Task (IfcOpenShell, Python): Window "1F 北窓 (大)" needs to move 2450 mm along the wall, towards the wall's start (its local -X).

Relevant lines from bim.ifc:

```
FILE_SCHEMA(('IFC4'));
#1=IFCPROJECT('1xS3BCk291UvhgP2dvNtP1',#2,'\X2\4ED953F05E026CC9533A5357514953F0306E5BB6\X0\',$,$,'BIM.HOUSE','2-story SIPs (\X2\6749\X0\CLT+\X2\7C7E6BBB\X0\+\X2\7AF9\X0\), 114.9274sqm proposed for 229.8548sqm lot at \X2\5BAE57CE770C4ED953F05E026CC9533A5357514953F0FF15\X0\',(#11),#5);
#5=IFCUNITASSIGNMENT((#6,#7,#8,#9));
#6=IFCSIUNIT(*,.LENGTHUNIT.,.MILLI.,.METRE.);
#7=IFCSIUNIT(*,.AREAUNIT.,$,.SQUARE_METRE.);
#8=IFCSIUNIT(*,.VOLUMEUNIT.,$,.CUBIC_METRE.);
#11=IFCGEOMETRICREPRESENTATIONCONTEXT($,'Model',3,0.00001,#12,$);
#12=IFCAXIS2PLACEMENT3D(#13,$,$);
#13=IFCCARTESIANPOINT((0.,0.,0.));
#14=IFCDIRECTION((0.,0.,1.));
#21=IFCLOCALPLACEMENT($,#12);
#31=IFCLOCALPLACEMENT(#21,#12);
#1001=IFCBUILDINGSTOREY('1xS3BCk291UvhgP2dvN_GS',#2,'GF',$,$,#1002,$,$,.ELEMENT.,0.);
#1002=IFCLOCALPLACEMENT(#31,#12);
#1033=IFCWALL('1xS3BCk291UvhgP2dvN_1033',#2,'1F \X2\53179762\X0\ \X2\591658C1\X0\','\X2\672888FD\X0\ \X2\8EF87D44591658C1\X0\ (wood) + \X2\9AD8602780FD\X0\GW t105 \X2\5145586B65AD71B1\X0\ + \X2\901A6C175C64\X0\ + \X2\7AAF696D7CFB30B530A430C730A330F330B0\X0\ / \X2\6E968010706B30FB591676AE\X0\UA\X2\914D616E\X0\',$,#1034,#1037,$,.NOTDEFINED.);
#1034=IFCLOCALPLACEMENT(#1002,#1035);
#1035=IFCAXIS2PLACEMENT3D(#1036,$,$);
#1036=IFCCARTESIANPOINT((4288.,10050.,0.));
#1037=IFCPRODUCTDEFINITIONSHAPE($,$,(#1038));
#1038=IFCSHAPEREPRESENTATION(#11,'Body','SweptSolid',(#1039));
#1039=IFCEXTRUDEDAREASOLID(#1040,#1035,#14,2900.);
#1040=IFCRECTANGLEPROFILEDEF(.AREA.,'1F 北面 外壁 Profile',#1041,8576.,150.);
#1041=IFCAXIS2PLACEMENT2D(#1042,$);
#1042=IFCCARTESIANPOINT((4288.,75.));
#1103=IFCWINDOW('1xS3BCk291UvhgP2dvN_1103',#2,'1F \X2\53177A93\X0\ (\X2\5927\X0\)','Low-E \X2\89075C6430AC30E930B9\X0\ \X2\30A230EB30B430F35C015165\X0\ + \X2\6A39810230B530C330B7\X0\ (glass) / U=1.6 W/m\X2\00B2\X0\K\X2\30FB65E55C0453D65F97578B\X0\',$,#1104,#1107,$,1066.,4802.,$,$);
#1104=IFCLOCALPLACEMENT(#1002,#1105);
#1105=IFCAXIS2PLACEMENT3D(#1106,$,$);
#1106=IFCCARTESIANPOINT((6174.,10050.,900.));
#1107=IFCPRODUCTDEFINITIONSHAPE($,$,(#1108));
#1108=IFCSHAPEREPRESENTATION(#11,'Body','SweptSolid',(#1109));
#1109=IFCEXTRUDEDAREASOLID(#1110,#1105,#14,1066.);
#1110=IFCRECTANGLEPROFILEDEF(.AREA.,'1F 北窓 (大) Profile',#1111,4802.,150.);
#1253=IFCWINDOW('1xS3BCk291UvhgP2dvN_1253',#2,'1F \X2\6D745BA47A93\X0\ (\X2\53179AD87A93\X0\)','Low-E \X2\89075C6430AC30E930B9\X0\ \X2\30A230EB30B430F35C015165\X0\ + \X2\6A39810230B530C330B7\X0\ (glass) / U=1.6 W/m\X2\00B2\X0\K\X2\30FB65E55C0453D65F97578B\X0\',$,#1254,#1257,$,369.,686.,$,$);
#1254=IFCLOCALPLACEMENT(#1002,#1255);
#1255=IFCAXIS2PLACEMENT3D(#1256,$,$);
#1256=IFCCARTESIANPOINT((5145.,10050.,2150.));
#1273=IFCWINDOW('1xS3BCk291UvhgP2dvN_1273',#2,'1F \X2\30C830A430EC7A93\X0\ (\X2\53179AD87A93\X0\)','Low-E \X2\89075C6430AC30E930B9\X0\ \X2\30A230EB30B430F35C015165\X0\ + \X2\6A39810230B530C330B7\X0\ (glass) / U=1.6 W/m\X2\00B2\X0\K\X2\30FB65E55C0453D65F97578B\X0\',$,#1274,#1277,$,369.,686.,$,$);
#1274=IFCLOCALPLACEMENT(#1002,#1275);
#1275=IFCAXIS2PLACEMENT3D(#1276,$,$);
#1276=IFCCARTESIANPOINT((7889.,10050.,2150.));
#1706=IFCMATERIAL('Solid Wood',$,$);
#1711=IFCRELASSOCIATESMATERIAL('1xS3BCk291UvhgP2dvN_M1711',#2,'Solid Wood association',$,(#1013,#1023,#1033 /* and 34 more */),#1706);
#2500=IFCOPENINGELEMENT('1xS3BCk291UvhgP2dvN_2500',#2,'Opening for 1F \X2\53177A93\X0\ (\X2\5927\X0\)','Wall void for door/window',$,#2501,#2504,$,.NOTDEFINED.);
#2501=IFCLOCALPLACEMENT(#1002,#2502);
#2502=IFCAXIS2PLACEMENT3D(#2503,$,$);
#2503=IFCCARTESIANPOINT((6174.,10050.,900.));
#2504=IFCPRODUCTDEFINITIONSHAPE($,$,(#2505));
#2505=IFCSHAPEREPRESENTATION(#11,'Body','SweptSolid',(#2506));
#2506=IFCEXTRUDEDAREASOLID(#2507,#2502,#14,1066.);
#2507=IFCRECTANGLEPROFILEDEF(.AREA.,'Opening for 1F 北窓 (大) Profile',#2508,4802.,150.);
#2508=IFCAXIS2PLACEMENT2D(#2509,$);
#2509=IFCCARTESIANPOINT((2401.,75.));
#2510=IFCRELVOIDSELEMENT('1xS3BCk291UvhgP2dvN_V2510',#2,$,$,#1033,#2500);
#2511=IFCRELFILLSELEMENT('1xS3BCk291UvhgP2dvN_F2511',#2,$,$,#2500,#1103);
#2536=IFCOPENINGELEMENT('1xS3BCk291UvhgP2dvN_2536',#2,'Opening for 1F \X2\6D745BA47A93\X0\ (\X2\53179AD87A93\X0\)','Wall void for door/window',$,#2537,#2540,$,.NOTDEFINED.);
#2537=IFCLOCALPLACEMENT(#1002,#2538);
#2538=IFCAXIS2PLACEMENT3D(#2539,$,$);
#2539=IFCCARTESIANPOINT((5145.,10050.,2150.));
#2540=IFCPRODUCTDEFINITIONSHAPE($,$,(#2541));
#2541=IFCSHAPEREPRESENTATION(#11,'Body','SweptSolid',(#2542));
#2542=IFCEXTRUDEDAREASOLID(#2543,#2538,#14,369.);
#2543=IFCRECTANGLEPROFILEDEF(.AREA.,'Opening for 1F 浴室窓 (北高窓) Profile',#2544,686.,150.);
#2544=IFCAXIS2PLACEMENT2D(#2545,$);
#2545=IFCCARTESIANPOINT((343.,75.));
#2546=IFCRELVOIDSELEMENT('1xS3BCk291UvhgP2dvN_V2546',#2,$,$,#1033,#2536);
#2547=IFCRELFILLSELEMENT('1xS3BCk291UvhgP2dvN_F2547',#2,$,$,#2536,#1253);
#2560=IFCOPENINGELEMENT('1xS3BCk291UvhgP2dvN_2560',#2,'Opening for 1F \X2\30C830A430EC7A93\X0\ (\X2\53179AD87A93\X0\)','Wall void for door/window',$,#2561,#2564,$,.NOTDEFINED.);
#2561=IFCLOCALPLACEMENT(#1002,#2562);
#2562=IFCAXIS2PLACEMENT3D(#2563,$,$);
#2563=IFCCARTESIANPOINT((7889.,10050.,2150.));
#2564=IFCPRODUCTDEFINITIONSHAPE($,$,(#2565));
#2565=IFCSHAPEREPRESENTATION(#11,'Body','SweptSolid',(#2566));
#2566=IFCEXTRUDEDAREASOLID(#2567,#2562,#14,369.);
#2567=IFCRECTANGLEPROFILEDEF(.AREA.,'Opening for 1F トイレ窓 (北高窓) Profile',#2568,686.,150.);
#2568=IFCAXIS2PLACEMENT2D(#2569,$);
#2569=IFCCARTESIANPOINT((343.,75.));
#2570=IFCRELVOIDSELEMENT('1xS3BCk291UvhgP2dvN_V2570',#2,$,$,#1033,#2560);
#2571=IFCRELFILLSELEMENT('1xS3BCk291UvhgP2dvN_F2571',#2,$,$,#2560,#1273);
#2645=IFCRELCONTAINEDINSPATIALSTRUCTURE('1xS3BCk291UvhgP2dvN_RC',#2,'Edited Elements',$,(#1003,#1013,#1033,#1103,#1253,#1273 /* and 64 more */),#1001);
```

```python
import ifcopenshell
import ifcopenshell.api.geometry
import ifcopenshell.util.placement

model = ifcopenshell.open("bim.ifc")

window = model.by_guid("1xS3BCk291UvhgP2dvN_1103")
opening = window.FillsVoids[0].RelatingOpeningElement
wall = opening.VoidsElements[0].RelatingBuildingElement

wall_matrix = ifcopenshell.util.placement.get_local_placement(wall.ObjectPlacement)
shift = wall_matrix[:3, 0] * -2450.0
before = ifcopenshell.util.placement.get_local_placement(window.ObjectPlacement)[:3, 3].copy()

# The window is not placed relative to its opening, so move both.
for product in (opening, window):
    matrix = ifcopenshell.util.placement.get_local_placement(product.ObjectPlacement)
    matrix[:3, 3] += shift
    ifcopenshell.api.geometry.edit_object_placement(model, product=product, matrix=matrix, is_si=False)

after = ifcopenshell.util.placement.get_local_placement(window.ObjectPlacement)[:3, 3]
print("window moved by", (after - before).round(3) + 0.0)

model.write("bim_v2.ifc")
```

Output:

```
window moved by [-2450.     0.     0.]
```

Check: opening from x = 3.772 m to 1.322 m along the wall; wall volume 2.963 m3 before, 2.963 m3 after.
